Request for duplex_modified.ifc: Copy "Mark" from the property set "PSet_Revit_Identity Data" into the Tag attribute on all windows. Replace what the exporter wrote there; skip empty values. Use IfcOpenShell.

First a look at what the model holds.

```python
import ifcopenshell
import ifcopenshell.util.element

model = ifcopenshell.open("duplex_modified.ifc")
print(model.schema)
windows = model.by_type("IfcWindow")
print(len(windows), "windows")
for e in windows[:8]:
    source = ifcopenshell.util.element.get_pset(e, "PSet_Revit_Identity Data", "Mark")
    target = e.Tag
    print(e.id(), repr(source), repr(target), sep=" | ")
```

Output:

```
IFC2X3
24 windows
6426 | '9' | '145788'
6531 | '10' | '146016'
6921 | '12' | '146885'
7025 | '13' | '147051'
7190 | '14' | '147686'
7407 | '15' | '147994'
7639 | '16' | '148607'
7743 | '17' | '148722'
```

```python
import ifcopenshell
import ifcopenshell.util.element

model = ifcopenshell.open("duplex_modified.ifc")

count = 0
for e in model.by_type("IfcWindow"):
    value = ifcopenshell.util.element.get_pset(e, "PSet_Revit_Identity Data", "Mark")
    current = e.Tag
    if not value or not value.strip() or current == value:
        continue
    e.Tag = value
    count += 1

print(count, "windows updated")

model.write("duplex_modified-out.ifc")
```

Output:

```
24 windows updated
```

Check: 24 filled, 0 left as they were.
